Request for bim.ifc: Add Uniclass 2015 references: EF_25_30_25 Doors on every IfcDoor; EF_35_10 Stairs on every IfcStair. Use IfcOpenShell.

First a look at what the model holds.

```python
import ifcopenshell

model = ifcopenshell.open("bim.ifc")
print(model.schema)
print("classifications:", [c.Name for c in model.by_type("IfcClassification")])
for ifc_class in ("IfcDoor", "IfcRoof", "IfcStair", "IfcWall", "IfcWindow"):
    print(ifc_class, len(model.by_type(ifc_class)))
```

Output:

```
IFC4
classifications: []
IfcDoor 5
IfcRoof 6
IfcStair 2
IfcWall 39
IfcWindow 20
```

```python
import ifcopenshell
import ifcopenshell.api.classification

model = ifcopenshell.open("bim.ifc")

system = ifcopenshell.api.classification.add_classification(model, classification="Uniclass 2015")

codes = {
    "IfcDoor": ("EF_25_30_25", "Doors"),
    "IfcStair": ("EF_35_10", "Stairs"),
}
for ifc_class, (code, name) in codes.items():
    products = model.by_type(ifc_class)
    ifcopenshell.api.classification.add_reference(
        model, products=products, classification=system, identification=code, name=name
    )
    print(code, len(products))

model.write("bim-out.ifc")
```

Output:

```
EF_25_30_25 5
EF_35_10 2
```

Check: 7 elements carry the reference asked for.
